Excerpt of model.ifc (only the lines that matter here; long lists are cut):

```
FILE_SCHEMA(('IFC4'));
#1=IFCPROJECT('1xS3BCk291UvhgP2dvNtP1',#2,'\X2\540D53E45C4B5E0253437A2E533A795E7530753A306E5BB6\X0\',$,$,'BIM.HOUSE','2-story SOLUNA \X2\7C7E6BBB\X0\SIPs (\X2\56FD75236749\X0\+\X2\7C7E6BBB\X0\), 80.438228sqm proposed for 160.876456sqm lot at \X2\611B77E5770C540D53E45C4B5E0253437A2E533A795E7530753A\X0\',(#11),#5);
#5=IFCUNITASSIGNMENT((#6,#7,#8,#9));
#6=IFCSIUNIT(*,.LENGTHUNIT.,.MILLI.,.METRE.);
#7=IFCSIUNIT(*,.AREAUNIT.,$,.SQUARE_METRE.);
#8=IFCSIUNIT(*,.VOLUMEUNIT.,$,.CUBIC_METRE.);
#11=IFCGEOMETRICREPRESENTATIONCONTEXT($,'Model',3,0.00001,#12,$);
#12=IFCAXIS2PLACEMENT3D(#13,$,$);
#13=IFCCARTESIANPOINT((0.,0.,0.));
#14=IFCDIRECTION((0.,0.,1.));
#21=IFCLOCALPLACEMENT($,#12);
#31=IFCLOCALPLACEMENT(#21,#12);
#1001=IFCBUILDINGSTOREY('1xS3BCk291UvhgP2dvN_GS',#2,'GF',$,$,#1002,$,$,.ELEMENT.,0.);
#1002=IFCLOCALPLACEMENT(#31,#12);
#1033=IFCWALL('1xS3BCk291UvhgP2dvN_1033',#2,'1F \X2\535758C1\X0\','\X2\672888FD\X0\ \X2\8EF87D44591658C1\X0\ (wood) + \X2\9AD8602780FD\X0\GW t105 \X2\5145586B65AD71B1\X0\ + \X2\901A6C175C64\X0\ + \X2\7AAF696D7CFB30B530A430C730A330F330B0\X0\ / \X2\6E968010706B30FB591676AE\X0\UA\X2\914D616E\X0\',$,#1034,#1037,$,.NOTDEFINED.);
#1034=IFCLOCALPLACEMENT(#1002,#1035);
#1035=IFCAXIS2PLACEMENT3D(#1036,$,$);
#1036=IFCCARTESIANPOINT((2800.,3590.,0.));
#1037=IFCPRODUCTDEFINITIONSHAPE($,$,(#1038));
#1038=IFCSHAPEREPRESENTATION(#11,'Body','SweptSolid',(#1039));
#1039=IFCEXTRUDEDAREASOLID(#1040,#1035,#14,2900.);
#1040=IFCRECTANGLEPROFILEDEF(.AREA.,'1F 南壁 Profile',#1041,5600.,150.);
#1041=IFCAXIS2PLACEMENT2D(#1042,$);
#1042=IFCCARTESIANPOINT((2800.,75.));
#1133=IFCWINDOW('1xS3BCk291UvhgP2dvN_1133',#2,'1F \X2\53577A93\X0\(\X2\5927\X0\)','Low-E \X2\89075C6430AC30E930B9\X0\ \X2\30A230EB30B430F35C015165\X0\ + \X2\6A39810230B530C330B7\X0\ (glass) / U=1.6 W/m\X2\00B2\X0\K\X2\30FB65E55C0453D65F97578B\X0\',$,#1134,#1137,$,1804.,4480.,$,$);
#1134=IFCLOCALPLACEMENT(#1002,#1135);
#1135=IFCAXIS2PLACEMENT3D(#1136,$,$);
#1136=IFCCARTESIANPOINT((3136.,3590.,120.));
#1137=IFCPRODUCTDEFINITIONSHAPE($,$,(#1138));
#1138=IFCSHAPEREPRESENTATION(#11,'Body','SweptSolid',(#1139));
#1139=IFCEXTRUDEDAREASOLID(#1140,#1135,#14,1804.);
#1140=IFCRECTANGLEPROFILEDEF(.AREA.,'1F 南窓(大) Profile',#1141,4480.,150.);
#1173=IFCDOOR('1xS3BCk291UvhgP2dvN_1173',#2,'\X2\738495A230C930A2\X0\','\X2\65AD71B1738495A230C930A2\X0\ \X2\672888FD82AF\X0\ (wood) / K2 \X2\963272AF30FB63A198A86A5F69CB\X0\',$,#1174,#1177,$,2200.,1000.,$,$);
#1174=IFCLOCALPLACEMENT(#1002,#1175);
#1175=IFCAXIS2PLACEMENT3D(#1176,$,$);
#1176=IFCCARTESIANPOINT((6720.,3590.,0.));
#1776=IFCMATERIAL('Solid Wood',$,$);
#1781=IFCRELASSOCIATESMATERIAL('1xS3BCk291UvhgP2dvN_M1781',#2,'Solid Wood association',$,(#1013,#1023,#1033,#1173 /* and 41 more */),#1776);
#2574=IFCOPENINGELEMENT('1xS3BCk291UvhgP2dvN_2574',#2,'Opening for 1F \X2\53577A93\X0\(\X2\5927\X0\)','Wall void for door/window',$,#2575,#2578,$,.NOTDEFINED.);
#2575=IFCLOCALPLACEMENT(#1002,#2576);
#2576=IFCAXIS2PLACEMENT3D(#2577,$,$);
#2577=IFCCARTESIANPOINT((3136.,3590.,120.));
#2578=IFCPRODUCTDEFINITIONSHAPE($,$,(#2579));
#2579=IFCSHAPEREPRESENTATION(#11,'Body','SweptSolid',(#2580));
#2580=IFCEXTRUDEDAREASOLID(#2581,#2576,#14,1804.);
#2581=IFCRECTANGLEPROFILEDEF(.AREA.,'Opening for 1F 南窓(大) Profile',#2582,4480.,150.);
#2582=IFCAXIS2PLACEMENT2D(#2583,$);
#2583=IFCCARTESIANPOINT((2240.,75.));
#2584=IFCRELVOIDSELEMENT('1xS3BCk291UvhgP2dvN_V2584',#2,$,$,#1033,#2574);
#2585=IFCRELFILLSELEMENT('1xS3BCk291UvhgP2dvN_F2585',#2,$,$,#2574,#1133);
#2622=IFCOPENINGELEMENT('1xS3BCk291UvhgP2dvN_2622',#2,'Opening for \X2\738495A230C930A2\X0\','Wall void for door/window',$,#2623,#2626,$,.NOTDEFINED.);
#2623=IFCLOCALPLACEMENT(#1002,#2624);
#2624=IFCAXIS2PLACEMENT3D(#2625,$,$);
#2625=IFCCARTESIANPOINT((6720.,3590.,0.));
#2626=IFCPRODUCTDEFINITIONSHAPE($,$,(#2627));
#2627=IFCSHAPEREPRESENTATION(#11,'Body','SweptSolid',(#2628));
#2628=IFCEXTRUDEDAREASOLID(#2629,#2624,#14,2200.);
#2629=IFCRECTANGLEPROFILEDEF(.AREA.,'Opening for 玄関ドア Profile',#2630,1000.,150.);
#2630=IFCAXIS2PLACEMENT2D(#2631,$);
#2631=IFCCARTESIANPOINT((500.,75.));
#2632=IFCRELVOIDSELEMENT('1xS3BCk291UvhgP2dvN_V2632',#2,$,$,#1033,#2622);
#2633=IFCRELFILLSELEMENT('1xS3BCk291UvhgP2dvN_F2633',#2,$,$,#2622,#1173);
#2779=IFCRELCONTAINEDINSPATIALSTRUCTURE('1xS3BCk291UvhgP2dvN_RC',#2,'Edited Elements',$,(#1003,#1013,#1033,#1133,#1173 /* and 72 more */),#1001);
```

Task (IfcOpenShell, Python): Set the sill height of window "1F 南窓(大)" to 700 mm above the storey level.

```python
import numpy as np
import ifcopenshell
import ifcopenshell.api.geometry
import ifcopenshell.geom
import ifcopenshell.util.element
import ifcopenshell.util.placement
import ifcopenshell.util.shape
import ifcopenshell.util.unit

model = ifcopenshell.open("model.ifc")
unit_scale = ifcopenshell.util.unit.calculate_unit_scale(model)

window = model.by_guid("1xS3BCk291UvhgP2dvN_1133")
opening = window.FillsVoids[0].RelatingOpeningElement
storey = ifcopenshell.util.element.get_container(window, ifc_class="IfcBuildingStorey")
level = ifcopenshell.util.placement.get_local_placement(storey.ObjectPlacement)[2, 3]

# The opening's origin need not be at the sill, so measure its lowest point.
shape = ifcopenshell.geom.create_shape(ifcopenshell.geom.settings(), opening)
bottom = ifcopenshell.util.shape.get_shape_bottom_elevation(shape, shape.geometry) / unit_scale
dz = level + 0.7 / unit_scale - bottom

shift = np.array([0.0, 0.0, dz])
# The window is not placed relative to its opening, so move both.
for product in (opening, window):
    matrix = ifcopenshell.util.placement.get_local_placement(product.ObjectPlacement)
    matrix[:3, 3] += shift
    ifcopenshell.api.geometry.edit_object_placement(model, product=product, matrix=matrix, is_si=False)

print(f"moved by {dz * unit_scale:+.3f} m")

model.write("model_v2.ifc")
```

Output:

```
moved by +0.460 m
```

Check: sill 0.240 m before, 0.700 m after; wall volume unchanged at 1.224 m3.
